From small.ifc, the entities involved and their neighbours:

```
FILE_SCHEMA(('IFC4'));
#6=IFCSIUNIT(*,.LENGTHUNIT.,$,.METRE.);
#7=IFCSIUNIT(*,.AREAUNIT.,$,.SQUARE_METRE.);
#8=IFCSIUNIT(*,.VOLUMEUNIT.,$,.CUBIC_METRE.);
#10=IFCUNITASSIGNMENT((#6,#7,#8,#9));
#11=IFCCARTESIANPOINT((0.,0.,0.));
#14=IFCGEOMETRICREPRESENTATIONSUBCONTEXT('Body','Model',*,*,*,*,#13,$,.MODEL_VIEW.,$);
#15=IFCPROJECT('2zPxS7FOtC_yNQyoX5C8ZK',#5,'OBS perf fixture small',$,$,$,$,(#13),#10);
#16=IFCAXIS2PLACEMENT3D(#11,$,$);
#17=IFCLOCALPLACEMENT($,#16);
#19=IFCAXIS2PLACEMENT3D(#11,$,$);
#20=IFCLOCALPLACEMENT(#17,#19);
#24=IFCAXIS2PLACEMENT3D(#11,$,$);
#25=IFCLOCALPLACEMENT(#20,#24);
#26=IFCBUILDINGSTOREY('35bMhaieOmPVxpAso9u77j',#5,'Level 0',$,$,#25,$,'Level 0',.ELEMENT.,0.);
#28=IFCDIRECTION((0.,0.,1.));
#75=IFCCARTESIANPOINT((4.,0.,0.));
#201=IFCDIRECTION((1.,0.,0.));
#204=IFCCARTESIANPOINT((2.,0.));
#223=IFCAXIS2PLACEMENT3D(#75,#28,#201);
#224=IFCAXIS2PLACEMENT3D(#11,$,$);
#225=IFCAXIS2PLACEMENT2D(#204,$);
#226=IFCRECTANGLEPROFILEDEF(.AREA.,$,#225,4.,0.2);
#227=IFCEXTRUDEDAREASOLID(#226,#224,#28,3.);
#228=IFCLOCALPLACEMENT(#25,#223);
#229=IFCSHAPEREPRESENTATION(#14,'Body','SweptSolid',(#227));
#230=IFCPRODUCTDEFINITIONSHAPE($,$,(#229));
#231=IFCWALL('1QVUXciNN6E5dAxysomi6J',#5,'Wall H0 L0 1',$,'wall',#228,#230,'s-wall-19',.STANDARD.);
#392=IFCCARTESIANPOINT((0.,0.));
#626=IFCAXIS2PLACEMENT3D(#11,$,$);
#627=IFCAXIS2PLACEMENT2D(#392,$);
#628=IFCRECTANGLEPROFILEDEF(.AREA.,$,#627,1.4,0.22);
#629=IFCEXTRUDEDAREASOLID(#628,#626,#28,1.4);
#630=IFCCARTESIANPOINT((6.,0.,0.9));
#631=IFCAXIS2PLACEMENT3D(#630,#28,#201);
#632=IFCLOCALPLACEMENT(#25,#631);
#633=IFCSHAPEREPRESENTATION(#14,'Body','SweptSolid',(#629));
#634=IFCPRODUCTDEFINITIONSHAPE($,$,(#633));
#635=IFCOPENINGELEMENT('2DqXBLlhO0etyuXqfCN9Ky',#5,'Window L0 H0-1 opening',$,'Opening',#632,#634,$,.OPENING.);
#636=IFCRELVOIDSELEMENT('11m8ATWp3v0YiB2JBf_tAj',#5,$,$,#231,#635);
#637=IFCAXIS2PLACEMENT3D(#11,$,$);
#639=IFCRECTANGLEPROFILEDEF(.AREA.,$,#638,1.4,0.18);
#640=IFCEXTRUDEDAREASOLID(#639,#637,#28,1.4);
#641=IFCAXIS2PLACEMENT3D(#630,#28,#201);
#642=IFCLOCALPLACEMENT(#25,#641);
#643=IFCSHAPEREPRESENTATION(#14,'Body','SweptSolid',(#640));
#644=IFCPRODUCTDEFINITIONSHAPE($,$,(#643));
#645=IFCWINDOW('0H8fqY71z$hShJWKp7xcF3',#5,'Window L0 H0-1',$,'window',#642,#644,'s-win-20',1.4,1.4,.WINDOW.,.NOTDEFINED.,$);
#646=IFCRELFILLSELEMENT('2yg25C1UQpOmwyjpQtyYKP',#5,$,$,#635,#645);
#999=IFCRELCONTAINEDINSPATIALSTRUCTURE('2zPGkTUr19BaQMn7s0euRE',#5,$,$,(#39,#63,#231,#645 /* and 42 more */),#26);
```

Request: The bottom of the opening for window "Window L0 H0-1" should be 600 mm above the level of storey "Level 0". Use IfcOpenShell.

```python
import numpy as np
import ifcopenshell
import ifcopenshell.api.geometry
import ifcopenshell.geom
import ifcopenshell.util.element
import ifcopenshell.util.placement
import ifcopenshell.util.shape
import ifcopenshell.util.unit

model = ifcopenshell.open("small.ifc")
unit_scale = ifcopenshell.util.unit.calculate_unit_scale(model)

window = model.by_guid("0H8fqY71z$hShJWKp7xcF3")
opening = window.FillsVoids[0].RelatingOpeningElement
storey = ifcopenshell.util.element.get_container(window, ifc_class="IfcBuildingStorey")
level = ifcopenshell.util.placement.get_local_placement(storey.ObjectPlacement)[2, 3]

# The opening's origin need not be at the sill, so measure its lowest point.
shape = ifcopenshell.geom.create_shape(ifcopenshell.geom.settings(), opening)
bottom = ifcopenshell.util.shape.get_shape_bottom_elevation(shape, shape.geometry) / unit_scale
dz = level + 0.6 - bottom

shift = np.array([0.0, 0.0, dz])
# The window is not placed relative to its opening, so move both.
for product in (opening, window):
    matrix = ifcopenshell.util.placement.get_local_placement(product.ObjectPlacement)
    matrix[:3, 3] += shift
    ifcopenshell.api.geometry.edit_object_placement(model, product=product, matrix=matrix, is_si=False)

print(f"moved by {dz * unit_scale:+.3f} m")

model.write("small_updated.ifc")
```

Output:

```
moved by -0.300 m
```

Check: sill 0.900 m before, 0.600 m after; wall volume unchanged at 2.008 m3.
